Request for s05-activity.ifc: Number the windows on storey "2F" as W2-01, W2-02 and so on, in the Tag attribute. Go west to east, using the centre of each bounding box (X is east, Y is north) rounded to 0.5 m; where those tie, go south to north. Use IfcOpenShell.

First a look at what the model holds.

```python
import ifcopenshell
import ifcopenshell.util.element
import ifcopenshell.util.placement

model = ifcopenshell.open("s05-activity.ifc")
print(model.schema)
storey = next(s for s in model.by_type("IfcBuildingStorey") if s.Name == "2F")
windows = [e for e in ifcopenshell.util.element.get_decomposition(storey) if e.is_a("IfcWindow")]
for e in sorted(windows, key=lambda e: e.id()):
    origin = ifcopenshell.util.placement.get_local_placement(e.ObjectPlacement)[:3, 3]
    print(e.id(), e.Tag, e.Name, origin.round(2) + 0.0, sep=" | ")
```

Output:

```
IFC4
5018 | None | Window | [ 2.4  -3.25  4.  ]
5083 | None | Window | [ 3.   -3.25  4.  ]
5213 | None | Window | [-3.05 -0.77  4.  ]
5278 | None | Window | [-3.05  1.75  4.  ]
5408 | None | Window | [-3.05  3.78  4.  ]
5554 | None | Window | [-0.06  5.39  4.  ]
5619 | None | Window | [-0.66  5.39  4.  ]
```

```python
import ifcopenshell
import ifcopenshell.geom
import ifcopenshell.util.element
import ifcopenshell.util.shape

model = ifcopenshell.open("s05-activity.ifc")
settings = ifcopenshell.geom.settings()
settings.set("use-world-coords", True)


def centre(element):
    shape = ifcopenshell.geom.create_shape(settings, element)
    return ifcopenshell.util.shape.get_bbox_centroid(shape.geometry)


storey = next(s for s in model.by_type("IfcBuildingStorey") if s.Name == "2F")
windows = [e for e in ifcopenshell.util.element.get_decomposition(storey) if e.is_a("IfcWindow")]

# Insertion points can sit at a corner or the storey origin, so sort by the geometry (in metres).
centres = {e: centre(e) for e in windows}
windows.sort(key=lambda e: (round(centres[e][0] / 0.5), centres[e][1]))

for i, e in enumerate(windows, start=1):
    number = f"W2-{i:02d}"
    e.Tag = number
    print(e.id(), number)

model.write("s05-activity-out.ifc")
```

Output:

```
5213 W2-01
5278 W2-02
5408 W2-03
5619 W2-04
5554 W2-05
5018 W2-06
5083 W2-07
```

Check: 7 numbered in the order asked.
